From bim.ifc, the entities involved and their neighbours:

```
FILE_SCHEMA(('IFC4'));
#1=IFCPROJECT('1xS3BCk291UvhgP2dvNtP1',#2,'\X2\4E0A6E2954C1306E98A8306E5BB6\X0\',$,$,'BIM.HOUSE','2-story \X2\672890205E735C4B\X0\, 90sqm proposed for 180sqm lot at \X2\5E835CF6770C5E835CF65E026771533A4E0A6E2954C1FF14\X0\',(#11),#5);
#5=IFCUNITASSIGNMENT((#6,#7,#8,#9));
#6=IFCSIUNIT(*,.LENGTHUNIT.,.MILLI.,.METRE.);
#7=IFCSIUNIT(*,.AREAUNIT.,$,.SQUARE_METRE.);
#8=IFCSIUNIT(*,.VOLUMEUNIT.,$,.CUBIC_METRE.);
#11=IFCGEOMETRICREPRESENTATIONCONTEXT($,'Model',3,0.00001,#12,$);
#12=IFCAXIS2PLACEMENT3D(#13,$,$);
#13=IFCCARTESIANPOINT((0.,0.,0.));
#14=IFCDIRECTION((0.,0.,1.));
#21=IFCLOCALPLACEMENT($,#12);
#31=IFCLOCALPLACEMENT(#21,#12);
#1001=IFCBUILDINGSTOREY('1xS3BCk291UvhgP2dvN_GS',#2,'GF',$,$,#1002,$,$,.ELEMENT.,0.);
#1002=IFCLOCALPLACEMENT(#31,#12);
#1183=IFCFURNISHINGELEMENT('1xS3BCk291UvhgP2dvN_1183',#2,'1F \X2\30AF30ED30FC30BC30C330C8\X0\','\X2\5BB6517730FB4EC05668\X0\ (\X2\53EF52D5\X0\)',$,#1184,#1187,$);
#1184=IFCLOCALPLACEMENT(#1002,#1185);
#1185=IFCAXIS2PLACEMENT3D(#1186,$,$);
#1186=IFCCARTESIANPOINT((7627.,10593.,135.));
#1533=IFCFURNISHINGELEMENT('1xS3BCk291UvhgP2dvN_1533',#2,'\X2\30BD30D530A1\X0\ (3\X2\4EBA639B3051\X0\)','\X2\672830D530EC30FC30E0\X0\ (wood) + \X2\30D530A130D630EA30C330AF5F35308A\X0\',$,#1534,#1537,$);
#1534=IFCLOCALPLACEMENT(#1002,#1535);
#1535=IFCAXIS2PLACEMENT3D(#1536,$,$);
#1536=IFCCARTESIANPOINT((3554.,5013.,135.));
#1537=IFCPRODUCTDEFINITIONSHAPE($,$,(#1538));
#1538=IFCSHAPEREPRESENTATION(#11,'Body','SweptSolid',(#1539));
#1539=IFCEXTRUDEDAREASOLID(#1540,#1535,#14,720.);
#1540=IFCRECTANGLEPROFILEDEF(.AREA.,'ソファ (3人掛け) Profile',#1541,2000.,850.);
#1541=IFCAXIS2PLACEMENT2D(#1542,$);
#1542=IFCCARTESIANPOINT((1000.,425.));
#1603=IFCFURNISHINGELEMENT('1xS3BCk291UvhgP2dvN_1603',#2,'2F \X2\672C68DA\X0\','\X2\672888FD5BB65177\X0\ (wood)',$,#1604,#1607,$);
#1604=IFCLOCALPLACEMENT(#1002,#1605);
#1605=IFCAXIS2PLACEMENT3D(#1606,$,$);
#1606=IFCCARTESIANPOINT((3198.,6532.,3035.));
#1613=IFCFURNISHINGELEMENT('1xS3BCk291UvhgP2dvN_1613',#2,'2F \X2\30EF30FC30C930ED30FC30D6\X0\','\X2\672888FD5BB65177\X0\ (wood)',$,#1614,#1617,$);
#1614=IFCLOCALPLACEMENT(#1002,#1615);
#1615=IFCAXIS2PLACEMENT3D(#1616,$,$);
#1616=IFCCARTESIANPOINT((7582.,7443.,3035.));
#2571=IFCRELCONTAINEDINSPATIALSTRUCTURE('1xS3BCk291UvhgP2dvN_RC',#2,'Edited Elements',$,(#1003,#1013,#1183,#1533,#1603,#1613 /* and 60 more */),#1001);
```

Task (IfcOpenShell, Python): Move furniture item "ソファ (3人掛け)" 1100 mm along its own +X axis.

```python
import ifcopenshell
import ifcopenshell.api.geometry
import ifcopenshell.util.placement
import ifcopenshell.util.unit

model = ifcopenshell.open("bim.ifc")
unit_scale = ifcopenshell.util.unit.calculate_unit_scale(model)

item = model.by_guid("1xS3BCk291UvhgP2dvN_1533")
matrix = ifcopenshell.util.placement.get_local_placement(item.ObjectPlacement)
matrix[:3, 3] += matrix[:3, 0] * 1.1 / unit_scale
ifcopenshell.api.geometry.edit_object_placement(model, product=item, matrix=matrix, is_si=False)

print(ifcopenshell.util.placement.get_local_placement(item.ObjectPlacement).round(3) + 0.0)

model.write("bim_edited.ifc")
```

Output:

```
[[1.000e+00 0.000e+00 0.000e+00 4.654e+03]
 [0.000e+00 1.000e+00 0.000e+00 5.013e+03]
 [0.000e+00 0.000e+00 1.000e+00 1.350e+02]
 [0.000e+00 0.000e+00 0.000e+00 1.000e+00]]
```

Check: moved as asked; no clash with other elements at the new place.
